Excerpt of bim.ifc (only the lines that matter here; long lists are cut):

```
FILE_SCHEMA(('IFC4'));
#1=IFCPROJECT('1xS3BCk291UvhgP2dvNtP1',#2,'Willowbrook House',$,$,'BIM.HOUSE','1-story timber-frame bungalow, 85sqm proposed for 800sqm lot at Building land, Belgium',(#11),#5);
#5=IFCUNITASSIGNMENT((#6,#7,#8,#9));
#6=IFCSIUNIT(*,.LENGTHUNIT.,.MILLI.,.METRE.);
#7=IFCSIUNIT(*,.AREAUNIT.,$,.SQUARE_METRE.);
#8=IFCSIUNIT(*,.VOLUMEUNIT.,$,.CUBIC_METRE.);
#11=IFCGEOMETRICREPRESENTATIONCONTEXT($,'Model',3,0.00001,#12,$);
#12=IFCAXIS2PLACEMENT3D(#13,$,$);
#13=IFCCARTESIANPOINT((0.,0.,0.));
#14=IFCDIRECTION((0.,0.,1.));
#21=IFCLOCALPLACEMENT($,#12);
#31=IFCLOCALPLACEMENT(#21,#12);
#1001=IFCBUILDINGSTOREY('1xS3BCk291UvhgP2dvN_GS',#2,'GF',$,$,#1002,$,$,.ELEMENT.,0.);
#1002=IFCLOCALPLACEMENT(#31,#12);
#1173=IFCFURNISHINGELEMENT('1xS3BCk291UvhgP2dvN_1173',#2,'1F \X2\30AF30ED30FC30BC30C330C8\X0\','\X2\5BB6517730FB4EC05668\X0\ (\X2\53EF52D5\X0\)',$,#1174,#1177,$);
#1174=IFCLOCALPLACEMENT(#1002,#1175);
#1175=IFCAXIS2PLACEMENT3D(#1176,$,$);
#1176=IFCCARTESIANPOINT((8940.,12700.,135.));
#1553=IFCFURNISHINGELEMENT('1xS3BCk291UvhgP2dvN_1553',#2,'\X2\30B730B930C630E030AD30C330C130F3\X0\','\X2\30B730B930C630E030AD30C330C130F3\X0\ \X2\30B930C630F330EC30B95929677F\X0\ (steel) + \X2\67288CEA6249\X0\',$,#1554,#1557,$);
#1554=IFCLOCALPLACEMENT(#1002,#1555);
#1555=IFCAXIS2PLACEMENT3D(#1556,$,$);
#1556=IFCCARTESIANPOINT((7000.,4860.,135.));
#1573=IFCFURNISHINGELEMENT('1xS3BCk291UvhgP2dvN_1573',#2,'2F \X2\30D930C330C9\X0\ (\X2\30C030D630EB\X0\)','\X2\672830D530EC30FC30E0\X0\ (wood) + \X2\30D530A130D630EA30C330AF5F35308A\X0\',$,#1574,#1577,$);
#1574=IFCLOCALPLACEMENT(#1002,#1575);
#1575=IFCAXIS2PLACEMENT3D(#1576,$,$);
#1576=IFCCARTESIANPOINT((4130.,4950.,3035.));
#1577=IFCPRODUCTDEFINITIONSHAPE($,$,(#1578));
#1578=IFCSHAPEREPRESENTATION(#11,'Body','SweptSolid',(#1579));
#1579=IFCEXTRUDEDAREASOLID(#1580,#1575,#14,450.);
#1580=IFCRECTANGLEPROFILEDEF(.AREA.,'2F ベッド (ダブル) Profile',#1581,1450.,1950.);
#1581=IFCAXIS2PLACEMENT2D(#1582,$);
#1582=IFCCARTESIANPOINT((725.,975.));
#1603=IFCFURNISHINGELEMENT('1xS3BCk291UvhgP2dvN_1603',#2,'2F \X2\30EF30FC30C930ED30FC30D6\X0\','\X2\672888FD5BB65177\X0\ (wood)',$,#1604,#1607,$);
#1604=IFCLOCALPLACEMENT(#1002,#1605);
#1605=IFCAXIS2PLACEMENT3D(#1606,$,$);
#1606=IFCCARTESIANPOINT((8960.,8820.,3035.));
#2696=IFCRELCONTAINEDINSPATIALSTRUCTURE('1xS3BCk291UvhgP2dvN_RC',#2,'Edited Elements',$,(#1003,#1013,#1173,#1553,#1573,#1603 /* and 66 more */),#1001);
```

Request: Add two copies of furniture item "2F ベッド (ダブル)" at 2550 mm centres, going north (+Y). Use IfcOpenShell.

```python
import numpy as np
import ifcopenshell
import ifcopenshell.api.geometry
import ifcopenshell.api.root
import ifcopenshell.util.element
import ifcopenshell.util.placement
import ifcopenshell.util.unit

model = ifcopenshell.open("bim.ifc")
unit_scale = ifcopenshell.util.unit.calculate_unit_scale(model)


def reuse_history(source, copy):
    """copy_class also copies each property set's owner history, people and application; keep the originals."""
    for rel in copy.IsDefinedBy:
        if rel.is_a("IfcRelDefinesByProperties") and (history := rel.RelatingPropertyDefinition.OwnerHistory):
            rel.RelatingPropertyDefinition.OwnerHistory = source.OwnerHistory
            ifcopenshell.util.element.remove_deep2(model, history)


source = model.by_guid("1xS3BCk291UvhgP2dvN_1573")
base = ifcopenshell.util.placement.get_local_placement(source.ObjectPlacement)
step = np.array([0.0, 1.0, 0.0]) * 2.55 / unit_scale

for i in range(1, 3):
    copy = ifcopenshell.api.root.copy_class(model, product=source)
    copy.Representation = ifcopenshell.util.element.copy_deep(
        model, source.Representation, exclude=["IfcGeometricRepresentationContext", "IfcRepresentationMap"]
    )
    reuse_history(source, copy)
    matrix = base.copy()
    matrix[:3, 3] += i * step
    print("added at", matrix[:3, 3].round(3) + 0.0)
    ifcopenshell.api.geometry.edit_object_placement(model, product=copy, matrix=matrix, is_si=False)

model.write("bim_updated.ifc")
```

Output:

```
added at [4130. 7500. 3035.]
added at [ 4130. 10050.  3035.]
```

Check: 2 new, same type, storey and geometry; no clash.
